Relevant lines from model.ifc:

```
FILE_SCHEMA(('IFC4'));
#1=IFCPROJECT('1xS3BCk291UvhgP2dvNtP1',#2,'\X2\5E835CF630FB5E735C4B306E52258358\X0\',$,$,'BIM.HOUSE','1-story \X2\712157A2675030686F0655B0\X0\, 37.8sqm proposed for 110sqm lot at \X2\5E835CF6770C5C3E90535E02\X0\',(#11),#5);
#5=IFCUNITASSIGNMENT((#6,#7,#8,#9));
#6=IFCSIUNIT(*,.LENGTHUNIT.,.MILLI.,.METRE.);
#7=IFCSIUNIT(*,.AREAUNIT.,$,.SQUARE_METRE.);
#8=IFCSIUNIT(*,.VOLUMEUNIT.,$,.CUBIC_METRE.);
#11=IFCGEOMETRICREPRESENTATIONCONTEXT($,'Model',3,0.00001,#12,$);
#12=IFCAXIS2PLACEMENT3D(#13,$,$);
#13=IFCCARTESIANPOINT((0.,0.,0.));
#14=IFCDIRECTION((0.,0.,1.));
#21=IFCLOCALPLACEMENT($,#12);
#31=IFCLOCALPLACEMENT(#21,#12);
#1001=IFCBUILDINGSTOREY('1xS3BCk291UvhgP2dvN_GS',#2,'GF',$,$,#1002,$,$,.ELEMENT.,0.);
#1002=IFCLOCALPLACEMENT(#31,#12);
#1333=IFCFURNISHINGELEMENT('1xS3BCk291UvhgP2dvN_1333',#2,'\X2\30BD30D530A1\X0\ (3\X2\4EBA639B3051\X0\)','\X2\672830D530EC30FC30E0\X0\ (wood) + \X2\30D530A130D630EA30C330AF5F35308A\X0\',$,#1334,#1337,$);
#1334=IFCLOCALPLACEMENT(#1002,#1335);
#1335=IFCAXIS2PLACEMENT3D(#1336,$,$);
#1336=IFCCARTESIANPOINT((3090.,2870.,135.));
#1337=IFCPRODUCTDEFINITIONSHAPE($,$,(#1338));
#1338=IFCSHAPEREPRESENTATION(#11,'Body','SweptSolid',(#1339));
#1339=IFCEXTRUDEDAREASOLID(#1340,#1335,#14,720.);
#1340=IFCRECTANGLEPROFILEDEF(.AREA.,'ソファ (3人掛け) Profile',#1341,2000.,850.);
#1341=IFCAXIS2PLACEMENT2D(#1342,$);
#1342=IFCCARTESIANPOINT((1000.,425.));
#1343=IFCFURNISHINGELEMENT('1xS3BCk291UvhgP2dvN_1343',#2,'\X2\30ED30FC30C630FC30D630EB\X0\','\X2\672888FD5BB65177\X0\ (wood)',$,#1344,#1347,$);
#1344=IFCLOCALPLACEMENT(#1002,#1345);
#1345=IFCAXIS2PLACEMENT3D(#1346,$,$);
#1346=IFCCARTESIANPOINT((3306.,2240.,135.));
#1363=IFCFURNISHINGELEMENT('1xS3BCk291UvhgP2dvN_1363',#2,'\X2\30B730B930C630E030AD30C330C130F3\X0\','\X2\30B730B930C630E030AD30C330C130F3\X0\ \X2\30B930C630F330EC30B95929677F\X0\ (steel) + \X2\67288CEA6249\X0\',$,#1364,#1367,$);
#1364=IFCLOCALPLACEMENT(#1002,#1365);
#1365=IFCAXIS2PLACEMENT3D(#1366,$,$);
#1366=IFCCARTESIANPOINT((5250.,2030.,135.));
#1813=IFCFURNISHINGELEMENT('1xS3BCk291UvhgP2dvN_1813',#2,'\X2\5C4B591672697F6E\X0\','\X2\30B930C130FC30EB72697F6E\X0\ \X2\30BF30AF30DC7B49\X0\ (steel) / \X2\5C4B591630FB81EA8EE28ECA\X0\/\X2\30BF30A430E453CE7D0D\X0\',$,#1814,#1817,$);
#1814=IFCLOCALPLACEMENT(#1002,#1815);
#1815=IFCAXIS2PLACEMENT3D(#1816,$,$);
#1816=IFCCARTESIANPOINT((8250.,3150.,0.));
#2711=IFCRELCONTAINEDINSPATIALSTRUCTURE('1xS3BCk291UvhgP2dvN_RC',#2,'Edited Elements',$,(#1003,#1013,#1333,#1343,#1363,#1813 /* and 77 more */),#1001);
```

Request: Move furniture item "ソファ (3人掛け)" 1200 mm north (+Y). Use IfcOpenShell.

```python
import ifcopenshell
import ifcopenshell.api.geometry
import ifcopenshell.util.placement

model = ifcopenshell.open("model.ifc")

item = model.by_guid("1xS3BCk291UvhgP2dvN_1333")
matrix = ifcopenshell.util.placement.get_local_placement(item.ObjectPlacement)
matrix[1, 3] += 1200.0
ifcopenshell.api.geometry.edit_object_placement(model, product=item, matrix=matrix, is_si=False)

print(ifcopenshell.util.placement.get_local_placement(item.ObjectPlacement).round(3) + 0.0)

model.write("model_v2.ifc")
```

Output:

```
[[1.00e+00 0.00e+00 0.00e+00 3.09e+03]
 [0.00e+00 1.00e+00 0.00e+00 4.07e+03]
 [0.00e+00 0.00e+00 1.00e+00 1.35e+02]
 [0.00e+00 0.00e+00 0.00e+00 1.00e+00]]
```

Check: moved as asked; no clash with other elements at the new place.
